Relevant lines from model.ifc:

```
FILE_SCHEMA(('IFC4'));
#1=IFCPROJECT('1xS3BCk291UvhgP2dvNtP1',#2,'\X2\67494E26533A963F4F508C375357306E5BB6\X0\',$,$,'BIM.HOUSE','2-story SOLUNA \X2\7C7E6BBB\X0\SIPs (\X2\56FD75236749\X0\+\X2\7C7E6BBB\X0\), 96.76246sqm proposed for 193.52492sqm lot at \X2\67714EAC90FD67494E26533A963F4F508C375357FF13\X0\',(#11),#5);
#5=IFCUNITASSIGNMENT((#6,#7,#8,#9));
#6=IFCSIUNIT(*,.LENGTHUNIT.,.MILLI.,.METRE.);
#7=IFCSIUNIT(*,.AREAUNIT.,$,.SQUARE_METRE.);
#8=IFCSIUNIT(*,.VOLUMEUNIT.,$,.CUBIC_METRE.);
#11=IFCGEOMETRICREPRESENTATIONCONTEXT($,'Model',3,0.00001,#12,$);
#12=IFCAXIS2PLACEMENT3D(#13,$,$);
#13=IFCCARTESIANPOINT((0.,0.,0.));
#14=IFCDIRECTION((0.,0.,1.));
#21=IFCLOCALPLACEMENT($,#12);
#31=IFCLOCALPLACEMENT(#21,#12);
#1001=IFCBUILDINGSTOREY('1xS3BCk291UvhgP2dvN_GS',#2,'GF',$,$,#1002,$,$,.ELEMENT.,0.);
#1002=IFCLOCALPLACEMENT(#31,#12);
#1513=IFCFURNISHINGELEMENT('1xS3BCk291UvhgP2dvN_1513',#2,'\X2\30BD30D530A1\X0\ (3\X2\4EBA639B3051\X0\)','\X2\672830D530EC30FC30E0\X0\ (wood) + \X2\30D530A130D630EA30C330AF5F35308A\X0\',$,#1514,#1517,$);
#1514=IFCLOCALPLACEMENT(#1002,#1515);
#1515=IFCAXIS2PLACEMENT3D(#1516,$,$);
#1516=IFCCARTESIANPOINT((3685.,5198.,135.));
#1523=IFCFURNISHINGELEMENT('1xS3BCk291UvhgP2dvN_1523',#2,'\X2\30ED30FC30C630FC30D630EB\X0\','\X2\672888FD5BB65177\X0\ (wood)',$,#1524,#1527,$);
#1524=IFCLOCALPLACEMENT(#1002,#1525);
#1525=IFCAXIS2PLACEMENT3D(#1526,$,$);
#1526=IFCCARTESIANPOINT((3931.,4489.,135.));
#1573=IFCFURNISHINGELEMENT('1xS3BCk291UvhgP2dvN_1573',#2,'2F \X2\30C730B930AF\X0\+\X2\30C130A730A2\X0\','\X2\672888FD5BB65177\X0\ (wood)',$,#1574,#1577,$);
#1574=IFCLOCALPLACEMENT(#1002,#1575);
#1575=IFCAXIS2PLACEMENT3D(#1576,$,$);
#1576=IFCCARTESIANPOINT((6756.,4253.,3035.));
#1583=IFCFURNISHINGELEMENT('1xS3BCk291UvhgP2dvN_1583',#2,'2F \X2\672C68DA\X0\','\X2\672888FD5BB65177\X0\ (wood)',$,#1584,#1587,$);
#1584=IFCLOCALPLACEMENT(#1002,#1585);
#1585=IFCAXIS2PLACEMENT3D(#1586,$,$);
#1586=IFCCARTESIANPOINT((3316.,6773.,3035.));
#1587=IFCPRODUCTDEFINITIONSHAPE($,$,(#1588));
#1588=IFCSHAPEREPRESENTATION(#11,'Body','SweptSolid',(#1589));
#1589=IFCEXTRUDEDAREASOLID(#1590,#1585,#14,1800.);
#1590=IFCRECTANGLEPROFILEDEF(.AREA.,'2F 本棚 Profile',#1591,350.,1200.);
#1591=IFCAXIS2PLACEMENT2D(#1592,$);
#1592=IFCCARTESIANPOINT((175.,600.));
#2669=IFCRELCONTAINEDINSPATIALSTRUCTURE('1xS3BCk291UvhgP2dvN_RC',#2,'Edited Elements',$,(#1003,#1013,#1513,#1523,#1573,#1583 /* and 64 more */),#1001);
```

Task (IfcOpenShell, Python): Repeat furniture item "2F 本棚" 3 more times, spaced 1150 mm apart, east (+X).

```python
import numpy as np
import ifcopenshell
import ifcopenshell.api.geometry
import ifcopenshell.api.root
import ifcopenshell.util.element
import ifcopenshell.util.placement
import ifcopenshell.util.unit

model = ifcopenshell.open("model.ifc")
unit_scale = ifcopenshell.util.unit.calculate_unit_scale(model)


def reuse_history(source, copy):
    """copy_class also copies each property set's owner history, people and application; keep the originals."""
    for rel in copy.IsDefinedBy:
        if rel.is_a("IfcRelDefinesByProperties") and (history := rel.RelatingPropertyDefinition.OwnerHistory):
            rel.RelatingPropertyDefinition.OwnerHistory = source.OwnerHistory
            ifcopenshell.util.element.remove_deep2(model, history)


source = model.by_guid("1xS3BCk291UvhgP2dvN_1583")
base = ifcopenshell.util.placement.get_local_placement(source.ObjectPlacement)
step = np.array([1.0, 0.0, 0.0]) * 1.15 / unit_scale

for i in range(1, 4):
    copy = ifcopenshell.api.root.copy_class(model, product=source)
    copy.Representation = ifcopenshell.util.element.copy_deep(
        model, source.Representation, exclude=["IfcGeometricRepresentationContext", "IfcRepresentationMap"]
    )
    reuse_history(source, copy)
    matrix = base.copy()
    matrix[:3, 3] += i * step
    print("added at", matrix[:3, 3].round(3) + 0.0)
    ifcopenshell.api.geometry.edit_object_placement(model, product=copy, matrix=matrix, is_si=False)

model.write("model_edited.ifc")
```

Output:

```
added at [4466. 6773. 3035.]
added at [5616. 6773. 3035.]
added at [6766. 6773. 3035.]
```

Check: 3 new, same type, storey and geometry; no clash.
